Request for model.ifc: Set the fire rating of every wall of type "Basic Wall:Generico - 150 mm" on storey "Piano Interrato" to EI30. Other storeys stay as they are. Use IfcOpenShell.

First a look at what the model holds.

```python
import ifcopenshell
import ifcopenshell.util.element

model = ifcopenshell.open("model.ifc")
print(model.schema)
storey = next(s for s in model.by_type("IfcBuildingStorey") if s.Name == "Piano Interrato")
walls = [e for e in ifcopenshell.util.element.get_decomposition(storey) if e.is_a("IfcWall")]
seen = {}
for e in walls:
    element_type = ifcopenshell.util.element.get_type(e)
    key = (element_type.Name if element_type != e and element_type else None, ifcopenshell.util.element.get_pset(e, "Pset_WallCommon", "FireRating"))
    seen[key] = seen.get(key, 0) + 1
for (name, value), count in sorted(seen.items(), key=str):
    print(count, "x", name, "|", value)
```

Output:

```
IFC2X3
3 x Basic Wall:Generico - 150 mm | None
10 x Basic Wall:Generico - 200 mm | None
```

```python
import ifcopenshell
import ifcopenshell.api.pset
import ifcopenshell.util.element

model = ifcopenshell.open("model.ifc")

storey = next(s for s in model.by_type("IfcBuildingStorey") if s.Name == "Piano Interrato")
walls = [e for e in ifcopenshell.util.element.get_decomposition(storey) if e.is_a("IfcWall")]

count = 0
for e in walls:
    element_type = ifcopenshell.util.element.get_type(e)
    if element_type in (None, e) or element_type.Name != "Basic Wall:Generico - 150 mm":
        continue
    # add_pset returns the element's existing set when there is one.
    pset = ifcopenshell.api.pset.add_pset(model, product=e, name="Pset_WallCommon")
    ifcopenshell.api.pset.edit_pset(model, pset=pset, properties={"FireRating": "EI30"})
    count += 1

print(count, "walls updated")

model.write("model_v2.ifc")
```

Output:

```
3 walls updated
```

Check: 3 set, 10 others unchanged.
